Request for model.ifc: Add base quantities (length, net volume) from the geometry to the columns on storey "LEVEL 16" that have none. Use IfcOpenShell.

First a look at what the model holds.

```python
import ifcopenshell
import ifcopenshell.util.element
import ifcopenshell.util.unit

model = ifcopenshell.open("model.ifc")
print(model.schema)
for unit_type in ("LENGTHUNIT", "AREAUNIT", "VOLUMEUNIT"):
    print(unit_type, ifcopenshell.util.unit.calculate_unit_scale(model, unit_type))
storey = next(s for s in model.by_type("IfcBuildingStorey") if s.Name == "LEVEL 16")
columns = [e for e in ifcopenshell.util.element.get_decomposition(storey) if e.is_a("IfcColumn")]
for e in sorted(columns, key=lambda e: e.id()):
    print(e.id(), e.is_a(), e.Name, list(ifcopenshell.util.element.get_psets(e, qtos_only=True)), sep=" | ")
```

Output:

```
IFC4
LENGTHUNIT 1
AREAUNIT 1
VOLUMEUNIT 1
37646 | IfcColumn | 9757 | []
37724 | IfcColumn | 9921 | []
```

```python
import ifcopenshell
import ifcopenshell.api.pset
import ifcopenshell.geom
import ifcopenshell.util.element
import ifcopenshell.util.shape
import ifcopenshell.util.unit

model = ifcopenshell.open("model.ifc")
unit_scale = ifcopenshell.util.unit.calculate_unit_scale(model)
volume_scale = ifcopenshell.util.unit.calculate_unit_scale(model, "VOLUMEUNIT")
settings = ifcopenshell.geom.settings()

storey = next(s for s in model.by_type("IfcBuildingStorey") if s.Name == "LEVEL 16")
columns = [e for e in ifcopenshell.util.element.get_decomposition(storey) if e.is_a("IfcColumn")]

for e in sorted(columns, key=lambda e: e.id()):
    if ifcopenshell.util.element.get_psets(e, qtos_only=True, should_inherit=False):
        continue
    # Geometry comes back in metres, in the element's own axes.
    shape = ifcopenshell.geom.create_shape(settings, e)
    values = {
        "Length": ifcopenshell.util.shape.get_z(shape.geometry) / unit_scale,
        "NetVolume": ifcopenshell.util.shape.get_volume(shape.geometry) / volume_scale,
    }
    qto = ifcopenshell.api.pset.add_qto(model, product=e, name="Qto_ColumnBaseQuantities")
    ifcopenshell.api.pset.edit_qto(model, qto=qto, properties=values)
    print(e.id(), {k: round(v, 3) for k, v in values.items()})

model.write("model_rev.ifc")
```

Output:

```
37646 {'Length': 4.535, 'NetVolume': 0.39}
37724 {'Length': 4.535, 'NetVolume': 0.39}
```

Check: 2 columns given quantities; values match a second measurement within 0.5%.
